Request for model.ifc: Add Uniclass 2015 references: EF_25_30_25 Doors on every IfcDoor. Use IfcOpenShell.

First a look at what the model holds.

```python
import ifcopenshell

model = ifcopenshell.open("model.ifc")
print(model.schema)
print("classifications:", [c.Name for c in model.by_type("IfcClassification")])
for ifc_class in ("IfcDoor", "IfcRoof", "IfcStair", "IfcWall", "IfcWindow"):
    print(ifc_class, len(model.by_type(ifc_class)))
```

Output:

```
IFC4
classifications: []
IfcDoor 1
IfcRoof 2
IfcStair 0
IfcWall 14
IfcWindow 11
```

```python
import ifcopenshell
import ifcopenshell.api.classification

model = ifcopenshell.open("model.ifc")

system = ifcopenshell.api.classification.add_classification(model, classification="Uniclass 2015")

codes = {
    "IfcDoor": ("EF_25_30_25", "Doors"),
}
for ifc_class, (code, name) in codes.items():
    products = model.by_type(ifc_class)
    ifcopenshell.api.classification.add_reference(
        model, products=products, classification=system, identification=code, name=name
    )
    print(code, len(products))

model.write("model_v2.ifc")
```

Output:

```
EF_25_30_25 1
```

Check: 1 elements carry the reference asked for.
